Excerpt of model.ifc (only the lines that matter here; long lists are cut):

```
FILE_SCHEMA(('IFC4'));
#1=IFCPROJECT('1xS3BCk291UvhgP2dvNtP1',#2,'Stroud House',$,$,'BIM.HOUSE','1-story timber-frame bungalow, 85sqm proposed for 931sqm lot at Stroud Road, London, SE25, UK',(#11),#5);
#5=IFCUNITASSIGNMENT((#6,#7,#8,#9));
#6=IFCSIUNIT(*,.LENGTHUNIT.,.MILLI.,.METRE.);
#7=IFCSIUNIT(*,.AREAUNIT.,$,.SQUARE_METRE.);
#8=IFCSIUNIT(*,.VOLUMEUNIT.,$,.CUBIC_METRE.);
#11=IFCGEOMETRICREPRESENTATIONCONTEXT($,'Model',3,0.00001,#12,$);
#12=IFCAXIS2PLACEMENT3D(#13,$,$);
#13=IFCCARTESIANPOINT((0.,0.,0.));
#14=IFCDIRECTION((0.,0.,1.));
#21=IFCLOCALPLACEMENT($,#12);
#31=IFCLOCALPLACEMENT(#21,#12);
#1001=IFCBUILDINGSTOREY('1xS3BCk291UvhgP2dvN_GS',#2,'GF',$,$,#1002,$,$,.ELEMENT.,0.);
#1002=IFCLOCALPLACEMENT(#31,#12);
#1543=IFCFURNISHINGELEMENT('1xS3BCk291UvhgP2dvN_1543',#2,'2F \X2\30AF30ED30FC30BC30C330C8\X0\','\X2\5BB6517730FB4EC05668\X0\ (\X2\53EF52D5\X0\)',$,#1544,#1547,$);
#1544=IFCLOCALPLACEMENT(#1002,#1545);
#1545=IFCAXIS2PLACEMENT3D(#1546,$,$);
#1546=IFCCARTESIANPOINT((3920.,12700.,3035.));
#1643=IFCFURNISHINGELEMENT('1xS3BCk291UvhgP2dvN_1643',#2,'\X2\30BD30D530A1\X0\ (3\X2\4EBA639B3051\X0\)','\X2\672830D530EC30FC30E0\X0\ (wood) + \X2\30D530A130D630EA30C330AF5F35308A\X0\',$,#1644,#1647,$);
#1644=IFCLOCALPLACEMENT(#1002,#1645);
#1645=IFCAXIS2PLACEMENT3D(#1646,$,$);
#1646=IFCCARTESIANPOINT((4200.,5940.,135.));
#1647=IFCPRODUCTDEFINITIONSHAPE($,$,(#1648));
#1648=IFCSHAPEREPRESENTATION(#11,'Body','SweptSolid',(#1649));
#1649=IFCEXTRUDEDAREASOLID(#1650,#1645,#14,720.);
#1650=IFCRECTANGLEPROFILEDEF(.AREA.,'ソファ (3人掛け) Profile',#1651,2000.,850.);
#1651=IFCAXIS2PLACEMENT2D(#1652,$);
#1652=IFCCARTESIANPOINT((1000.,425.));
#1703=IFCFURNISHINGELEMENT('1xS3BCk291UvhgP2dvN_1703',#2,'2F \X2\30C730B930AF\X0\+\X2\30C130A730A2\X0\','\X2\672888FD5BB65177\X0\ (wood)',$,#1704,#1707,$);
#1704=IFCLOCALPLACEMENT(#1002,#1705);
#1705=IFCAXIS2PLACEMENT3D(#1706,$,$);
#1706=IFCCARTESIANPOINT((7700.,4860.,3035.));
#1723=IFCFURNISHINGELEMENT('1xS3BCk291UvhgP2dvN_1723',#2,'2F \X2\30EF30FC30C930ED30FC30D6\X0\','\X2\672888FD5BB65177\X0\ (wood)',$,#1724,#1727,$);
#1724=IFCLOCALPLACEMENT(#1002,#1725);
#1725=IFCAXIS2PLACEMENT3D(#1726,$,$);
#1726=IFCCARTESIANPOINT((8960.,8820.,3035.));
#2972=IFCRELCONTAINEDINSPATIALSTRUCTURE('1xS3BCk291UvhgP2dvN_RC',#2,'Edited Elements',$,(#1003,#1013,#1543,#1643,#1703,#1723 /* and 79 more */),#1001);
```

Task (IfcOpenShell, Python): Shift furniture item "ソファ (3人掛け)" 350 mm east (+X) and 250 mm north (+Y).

```python
import ifcopenshell
import ifcopenshell.api.geometry
import ifcopenshell.util.placement

model = ifcopenshell.open("model.ifc")

item = model.by_guid("1xS3BCk291UvhgP2dvN_1643")
matrix = ifcopenshell.util.placement.get_local_placement(item.ObjectPlacement)
matrix[0, 3] += 350.0
matrix[1, 3] += 250.0
ifcopenshell.api.geometry.edit_object_placement(model, product=item, matrix=matrix, is_si=False)

print(ifcopenshell.util.placement.get_local_placement(item.ObjectPlacement).round(3) + 0.0)

model.write("model_v2.ifc")
```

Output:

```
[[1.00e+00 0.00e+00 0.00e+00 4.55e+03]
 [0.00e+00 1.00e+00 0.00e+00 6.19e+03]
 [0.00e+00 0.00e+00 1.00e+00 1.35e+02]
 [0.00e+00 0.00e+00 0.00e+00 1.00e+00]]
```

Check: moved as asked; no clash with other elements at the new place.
